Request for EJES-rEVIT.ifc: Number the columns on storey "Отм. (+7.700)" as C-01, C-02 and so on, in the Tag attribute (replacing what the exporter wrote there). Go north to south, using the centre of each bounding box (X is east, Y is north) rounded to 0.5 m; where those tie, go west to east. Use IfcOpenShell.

First a look at what the model holds.

```python
import ifcopenshell
import ifcopenshell.util.element
import ifcopenshell.util.placement

model = ifcopenshell.open("EJES-rEVIT.ifc")
print(model.schema)
storey = next(s for s in model.by_type("IfcBuildingStorey") if s.Name == "Отм. (+7.700)")
columns = [e for e in ifcopenshell.util.element.get_decomposition(storey) if e.is_a("IfcColumn")]
for e in sorted(columns, key=lambda e: e.id()):
    origin = ifcopenshell.util.placement.get_local_placement(e.ObjectPlacement)[:3, 3]
    print(e.id(), e.Tag, e.Name, origin.round(2) + 0.0, sep=" | ")
```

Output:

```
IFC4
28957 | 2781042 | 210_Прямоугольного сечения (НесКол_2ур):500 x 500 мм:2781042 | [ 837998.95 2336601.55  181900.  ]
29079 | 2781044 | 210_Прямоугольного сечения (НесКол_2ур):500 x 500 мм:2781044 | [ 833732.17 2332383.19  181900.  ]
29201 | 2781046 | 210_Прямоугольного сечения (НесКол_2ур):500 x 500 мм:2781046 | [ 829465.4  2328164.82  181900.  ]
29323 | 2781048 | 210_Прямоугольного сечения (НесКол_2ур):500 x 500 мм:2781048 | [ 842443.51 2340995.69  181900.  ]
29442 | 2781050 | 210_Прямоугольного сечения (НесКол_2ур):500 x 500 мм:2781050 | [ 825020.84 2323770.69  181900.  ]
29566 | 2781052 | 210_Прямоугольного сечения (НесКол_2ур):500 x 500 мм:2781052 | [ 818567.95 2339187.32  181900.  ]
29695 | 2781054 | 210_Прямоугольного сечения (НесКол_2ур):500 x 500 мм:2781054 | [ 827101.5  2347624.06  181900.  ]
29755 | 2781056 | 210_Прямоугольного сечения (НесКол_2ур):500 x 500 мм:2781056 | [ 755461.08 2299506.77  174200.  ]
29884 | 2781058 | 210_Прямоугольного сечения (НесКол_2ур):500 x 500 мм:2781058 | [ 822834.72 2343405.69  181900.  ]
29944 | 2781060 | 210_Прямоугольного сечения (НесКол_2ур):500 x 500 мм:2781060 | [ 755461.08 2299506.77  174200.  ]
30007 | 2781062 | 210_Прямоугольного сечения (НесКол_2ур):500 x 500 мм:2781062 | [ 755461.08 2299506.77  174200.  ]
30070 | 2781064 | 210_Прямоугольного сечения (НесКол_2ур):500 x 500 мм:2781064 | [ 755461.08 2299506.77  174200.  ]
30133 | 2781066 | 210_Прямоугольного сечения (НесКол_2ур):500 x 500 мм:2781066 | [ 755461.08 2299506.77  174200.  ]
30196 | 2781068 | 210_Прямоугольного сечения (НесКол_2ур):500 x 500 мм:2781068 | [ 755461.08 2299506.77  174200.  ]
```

```python
import ifcopenshell
import ifcopenshell.geom
import ifcopenshell.util.element
import ifcopenshell.util.shape

model = ifcopenshell.open("EJES-rEVIT.ifc")
settings = ifcopenshell.geom.settings()
settings.set("use-world-coords", True)


def centre(element):
    shape = ifcopenshell.geom.create_shape(settings, element)
    return ifcopenshell.util.shape.get_bbox_centroid(shape.geometry)


storey = next(s for s in model.by_type("IfcBuildingStorey") if s.Name == "Отм. (+7.700)")
columns = [e for e in ifcopenshell.util.element.get_decomposition(storey) if e.is_a("IfcColumn")]

# Insertion points can sit at a corner or the storey origin, so sort by the geometry (in metres).
centres = {e: centre(e) for e in columns}
columns.sort(key=lambda e: (-round(centres[e][1] / 0.5), centres[e][0]))

for i, e in enumerate(columns, start=1):
    number = f"C-{i:02d}"
    e.Tag = number
    print(e.id(), number)

model.write("EJES-rEVIT_edited.ifc")
```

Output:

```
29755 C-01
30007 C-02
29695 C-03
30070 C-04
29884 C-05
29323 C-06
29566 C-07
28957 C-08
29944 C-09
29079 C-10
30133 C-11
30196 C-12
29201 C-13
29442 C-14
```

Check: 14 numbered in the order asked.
